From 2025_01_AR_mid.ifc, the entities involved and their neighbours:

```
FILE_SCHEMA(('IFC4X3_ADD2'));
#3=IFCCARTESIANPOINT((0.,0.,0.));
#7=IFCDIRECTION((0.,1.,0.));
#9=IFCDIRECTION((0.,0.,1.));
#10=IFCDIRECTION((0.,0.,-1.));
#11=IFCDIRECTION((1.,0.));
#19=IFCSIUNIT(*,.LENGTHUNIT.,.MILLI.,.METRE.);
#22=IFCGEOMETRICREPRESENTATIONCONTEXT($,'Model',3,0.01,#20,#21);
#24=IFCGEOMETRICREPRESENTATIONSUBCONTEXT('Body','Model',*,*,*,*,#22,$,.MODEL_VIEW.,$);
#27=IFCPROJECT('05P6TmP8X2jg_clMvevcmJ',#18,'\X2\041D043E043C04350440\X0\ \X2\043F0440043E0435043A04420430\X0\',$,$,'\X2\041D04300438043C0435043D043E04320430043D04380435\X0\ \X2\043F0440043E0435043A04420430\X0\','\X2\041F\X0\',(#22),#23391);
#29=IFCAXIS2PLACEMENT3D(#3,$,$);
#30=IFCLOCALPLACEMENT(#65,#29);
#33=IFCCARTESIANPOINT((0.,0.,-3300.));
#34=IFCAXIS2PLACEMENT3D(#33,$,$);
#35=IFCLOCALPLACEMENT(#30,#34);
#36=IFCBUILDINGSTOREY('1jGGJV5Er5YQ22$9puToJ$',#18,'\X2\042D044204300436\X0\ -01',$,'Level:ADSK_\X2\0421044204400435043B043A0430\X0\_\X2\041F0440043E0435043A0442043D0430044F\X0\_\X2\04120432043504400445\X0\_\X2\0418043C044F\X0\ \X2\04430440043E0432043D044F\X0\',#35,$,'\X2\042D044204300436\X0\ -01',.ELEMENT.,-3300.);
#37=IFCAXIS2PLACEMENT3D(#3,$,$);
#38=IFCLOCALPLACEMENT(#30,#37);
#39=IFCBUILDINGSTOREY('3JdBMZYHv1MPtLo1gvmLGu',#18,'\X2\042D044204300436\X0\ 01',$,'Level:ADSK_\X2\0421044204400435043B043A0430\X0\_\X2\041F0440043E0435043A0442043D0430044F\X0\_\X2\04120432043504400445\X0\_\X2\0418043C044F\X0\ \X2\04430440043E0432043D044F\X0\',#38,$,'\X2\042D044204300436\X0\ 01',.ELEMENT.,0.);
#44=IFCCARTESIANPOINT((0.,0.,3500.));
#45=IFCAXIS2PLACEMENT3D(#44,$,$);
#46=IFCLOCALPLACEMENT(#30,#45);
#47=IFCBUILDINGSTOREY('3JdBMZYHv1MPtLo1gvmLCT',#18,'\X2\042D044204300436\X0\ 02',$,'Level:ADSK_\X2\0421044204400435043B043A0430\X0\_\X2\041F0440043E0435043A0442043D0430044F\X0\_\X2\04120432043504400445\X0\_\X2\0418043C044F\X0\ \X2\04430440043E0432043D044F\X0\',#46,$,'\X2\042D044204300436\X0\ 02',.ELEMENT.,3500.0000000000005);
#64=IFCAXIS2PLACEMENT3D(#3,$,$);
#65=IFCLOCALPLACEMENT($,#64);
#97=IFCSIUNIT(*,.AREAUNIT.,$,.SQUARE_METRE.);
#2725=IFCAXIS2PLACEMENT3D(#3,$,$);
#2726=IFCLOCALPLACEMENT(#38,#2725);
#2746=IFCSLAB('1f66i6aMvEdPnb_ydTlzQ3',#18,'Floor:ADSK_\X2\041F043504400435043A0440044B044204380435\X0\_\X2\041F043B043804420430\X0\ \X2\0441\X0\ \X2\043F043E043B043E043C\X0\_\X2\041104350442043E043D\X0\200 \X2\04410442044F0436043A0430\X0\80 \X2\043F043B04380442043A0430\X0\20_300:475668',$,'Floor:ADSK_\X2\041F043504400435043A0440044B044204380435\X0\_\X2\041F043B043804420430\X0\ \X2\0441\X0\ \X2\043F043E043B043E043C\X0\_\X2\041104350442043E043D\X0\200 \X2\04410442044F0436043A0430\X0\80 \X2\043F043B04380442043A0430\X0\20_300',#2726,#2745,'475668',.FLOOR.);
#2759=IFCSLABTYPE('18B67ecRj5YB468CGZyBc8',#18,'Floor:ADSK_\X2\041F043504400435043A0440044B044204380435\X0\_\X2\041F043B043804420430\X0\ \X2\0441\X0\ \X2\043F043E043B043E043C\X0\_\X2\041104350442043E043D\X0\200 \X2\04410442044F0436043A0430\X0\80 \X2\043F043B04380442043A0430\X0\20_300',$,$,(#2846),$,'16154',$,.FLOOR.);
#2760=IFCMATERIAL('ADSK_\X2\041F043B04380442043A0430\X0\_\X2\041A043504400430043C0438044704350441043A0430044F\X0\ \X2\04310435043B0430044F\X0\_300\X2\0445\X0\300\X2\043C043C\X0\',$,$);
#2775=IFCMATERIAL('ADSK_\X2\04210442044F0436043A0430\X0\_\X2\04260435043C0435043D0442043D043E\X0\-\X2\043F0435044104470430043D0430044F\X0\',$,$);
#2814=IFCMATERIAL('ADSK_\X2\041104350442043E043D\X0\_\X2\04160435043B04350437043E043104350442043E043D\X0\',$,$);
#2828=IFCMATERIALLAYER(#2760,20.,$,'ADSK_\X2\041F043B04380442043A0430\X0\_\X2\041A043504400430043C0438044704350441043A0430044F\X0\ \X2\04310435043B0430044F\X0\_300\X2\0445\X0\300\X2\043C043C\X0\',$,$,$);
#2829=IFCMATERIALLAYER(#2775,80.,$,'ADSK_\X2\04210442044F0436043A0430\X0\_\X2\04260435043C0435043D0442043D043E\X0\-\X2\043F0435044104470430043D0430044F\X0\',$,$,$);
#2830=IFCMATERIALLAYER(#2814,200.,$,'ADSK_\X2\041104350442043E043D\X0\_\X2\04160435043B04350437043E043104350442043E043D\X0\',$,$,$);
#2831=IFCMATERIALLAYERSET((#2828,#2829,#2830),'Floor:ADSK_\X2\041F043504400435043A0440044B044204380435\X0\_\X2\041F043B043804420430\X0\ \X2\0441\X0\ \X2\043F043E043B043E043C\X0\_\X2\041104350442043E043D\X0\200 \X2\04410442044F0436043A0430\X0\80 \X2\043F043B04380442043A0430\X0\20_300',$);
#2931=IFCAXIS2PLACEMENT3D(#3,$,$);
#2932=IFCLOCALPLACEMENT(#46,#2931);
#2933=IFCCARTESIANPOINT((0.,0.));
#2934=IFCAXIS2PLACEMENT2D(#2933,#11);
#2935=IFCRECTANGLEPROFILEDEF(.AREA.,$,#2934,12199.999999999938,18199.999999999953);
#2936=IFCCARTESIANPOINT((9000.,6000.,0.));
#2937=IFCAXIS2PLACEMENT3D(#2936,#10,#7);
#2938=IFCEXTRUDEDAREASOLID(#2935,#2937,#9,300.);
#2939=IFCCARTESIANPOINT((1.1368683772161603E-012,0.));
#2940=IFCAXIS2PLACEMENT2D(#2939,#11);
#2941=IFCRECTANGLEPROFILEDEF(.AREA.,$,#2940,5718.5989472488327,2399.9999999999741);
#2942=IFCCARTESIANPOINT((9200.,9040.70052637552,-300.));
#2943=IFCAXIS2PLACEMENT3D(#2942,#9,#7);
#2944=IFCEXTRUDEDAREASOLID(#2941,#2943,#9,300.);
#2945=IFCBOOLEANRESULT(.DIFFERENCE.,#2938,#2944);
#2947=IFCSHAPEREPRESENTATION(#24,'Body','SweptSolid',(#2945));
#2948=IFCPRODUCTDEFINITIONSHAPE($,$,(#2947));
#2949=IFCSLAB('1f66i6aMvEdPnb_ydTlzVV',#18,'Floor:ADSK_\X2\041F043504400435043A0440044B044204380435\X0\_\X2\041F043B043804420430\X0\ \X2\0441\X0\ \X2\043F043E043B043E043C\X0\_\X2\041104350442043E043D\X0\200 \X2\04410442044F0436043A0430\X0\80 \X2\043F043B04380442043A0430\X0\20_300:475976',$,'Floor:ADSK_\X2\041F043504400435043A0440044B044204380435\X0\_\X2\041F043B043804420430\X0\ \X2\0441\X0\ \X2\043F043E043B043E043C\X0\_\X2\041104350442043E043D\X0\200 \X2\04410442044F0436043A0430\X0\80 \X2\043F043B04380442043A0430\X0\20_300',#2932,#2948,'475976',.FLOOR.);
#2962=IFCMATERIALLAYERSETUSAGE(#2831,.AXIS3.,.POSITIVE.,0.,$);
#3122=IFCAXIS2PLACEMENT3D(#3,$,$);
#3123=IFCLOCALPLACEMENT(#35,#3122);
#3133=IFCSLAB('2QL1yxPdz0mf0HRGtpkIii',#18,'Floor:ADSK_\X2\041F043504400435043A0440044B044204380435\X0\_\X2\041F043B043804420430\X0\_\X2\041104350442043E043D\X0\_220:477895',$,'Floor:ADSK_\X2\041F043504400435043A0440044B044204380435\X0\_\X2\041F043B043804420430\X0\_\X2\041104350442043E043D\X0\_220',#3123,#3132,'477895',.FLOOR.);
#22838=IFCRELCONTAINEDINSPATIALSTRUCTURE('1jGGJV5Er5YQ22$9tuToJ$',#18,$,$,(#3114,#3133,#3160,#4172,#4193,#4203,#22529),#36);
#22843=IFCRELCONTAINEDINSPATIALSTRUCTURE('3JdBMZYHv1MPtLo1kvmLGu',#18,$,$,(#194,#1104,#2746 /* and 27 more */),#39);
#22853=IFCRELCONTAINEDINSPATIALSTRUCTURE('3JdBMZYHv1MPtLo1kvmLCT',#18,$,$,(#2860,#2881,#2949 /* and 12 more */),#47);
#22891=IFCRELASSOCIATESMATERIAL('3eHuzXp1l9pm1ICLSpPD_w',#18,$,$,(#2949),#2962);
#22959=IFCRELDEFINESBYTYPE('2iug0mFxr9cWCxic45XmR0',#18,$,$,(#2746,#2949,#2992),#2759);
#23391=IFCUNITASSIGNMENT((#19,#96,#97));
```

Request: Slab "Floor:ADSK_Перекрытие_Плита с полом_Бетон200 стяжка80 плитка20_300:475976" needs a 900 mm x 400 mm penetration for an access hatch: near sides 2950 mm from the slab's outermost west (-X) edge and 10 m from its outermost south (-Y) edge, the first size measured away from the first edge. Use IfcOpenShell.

```python
import numpy as np
import ifcopenshell
import ifcopenshell.api.feature
import ifcopenshell.api.geometry
import ifcopenshell.api.root
import ifcopenshell.geom
import ifcopenshell.util.placement
import ifcopenshell.util.representation
import ifcopenshell.util.shape
import ifcopenshell.util.unit

model = ifcopenshell.open("2025_01_AR_mid.ifc")
unit_scale = ifcopenshell.util.unit.calculate_unit_scale(model)
settings = ifcopenshell.geom.settings()


def volume(element):
    """Net volume in cubic metres, openings subtracted."""
    shape = ifcopenshell.geom.create_shape(settings, element)
    return ifcopenshell.util.shape.get_volume(shape.geometry)


slab = model.by_id(2949)
before = volume(slab)

# Extent in the slab's own axes, in metres. The edges named are its -X and -Y sides.
slab_shape = ifcopenshell.geom.create_shape(settings, slab)
vertices = ifcopenshell.util.shape.get_vertices(slab_shape.geometry)
x_min, y_min, bottom = vertices.min(axis=0)
top = vertices[:, 2].max()

opening = ifcopenshell.api.root.create_entity(model, ifc_class="IfcOpeningElement", name="Access hatch opening", predefined_type="OPENING")
context = ifcopenshell.util.representation.get_context(model, "Model", "Body", "MODEL_VIEW")
width, depth = 0.9, 0.4
outline = [(0.0, 0.0), (width, 0.0), (width, depth), (0.0, depth), (0.0, 0.0)]
# Overshoot both faces by 50 mm so the cut is clean.
shape = ifcopenshell.api.geometry.add_slab_representation(
    model, context=context, depth=top - bottom + 0.1, polyline=outline
)
ifcopenshell.api.geometry.assign_representation(model, product=opening, representation=shape)

matrix = ifcopenshell.util.placement.get_local_placement(slab.ObjectPlacement)
matrix[:, 3] = matrix @ np.append(np.array([x_min + 2.95, y_min + 10, bottom - 0.05]) / unit_scale, 1.0)
ifcopenshell.api.geometry.edit_object_placement(model, product=opening, matrix=matrix, is_si=False)
ifcopenshell.api.feature.add_feature(model, feature=opening, element=slab)

after = volume(slab)

print(f"slab volume {before:.3f} -> {after:.3f} m3")

model.write("2025_01_AR_mid_v2.ifc")
```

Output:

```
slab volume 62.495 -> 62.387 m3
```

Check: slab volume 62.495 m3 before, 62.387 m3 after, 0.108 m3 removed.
